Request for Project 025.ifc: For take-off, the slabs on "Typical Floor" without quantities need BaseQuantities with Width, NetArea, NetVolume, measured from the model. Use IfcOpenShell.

First a look at what the model holds.

```python
import ifcopenshell
import ifcopenshell.util.element
import ifcopenshell.util.unit

model = ifcopenshell.open("Project 025.ifc")
print(model.schema)
for unit_type in ("LENGTHUNIT", "AREAUNIT", "VOLUMEUNIT"):
    print(unit_type, ifcopenshell.util.unit.calculate_unit_scale(model, unit_type))
storey = next(s for s in model.by_type("IfcBuildingStorey") if s.Name == "Typical Floor")
slabs = [e for e in ifcopenshell.util.element.get_decomposition(storey) if e.is_a("IfcSlab")]
for e in sorted(slabs, key=lambda e: e.id()):
    print(e.id(), e.is_a(), e.Name, list(ifcopenshell.util.element.get_psets(e, qtos_only=True)), sep=" | ")
```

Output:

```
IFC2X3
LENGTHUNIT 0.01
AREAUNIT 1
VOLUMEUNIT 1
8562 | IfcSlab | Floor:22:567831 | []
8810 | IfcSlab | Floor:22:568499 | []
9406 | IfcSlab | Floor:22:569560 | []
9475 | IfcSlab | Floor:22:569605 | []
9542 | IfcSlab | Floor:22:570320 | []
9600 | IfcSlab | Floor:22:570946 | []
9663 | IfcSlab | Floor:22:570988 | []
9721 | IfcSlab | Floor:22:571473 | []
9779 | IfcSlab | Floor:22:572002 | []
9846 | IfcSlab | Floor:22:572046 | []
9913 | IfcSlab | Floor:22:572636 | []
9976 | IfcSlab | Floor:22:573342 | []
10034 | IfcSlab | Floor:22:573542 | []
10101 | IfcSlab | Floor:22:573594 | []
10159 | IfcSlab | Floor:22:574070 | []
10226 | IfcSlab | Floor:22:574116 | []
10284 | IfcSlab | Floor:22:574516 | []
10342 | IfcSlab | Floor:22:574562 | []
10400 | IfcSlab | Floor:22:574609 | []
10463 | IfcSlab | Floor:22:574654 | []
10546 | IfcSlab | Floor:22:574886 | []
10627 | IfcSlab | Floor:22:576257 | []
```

```python
import ifcopenshell
import ifcopenshell.api.pset
import ifcopenshell.geom
import ifcopenshell.util.element
import ifcopenshell.util.shape
import ifcopenshell.util.unit

model = ifcopenshell.open("Project 025.ifc")
unit_scale = ifcopenshell.util.unit.calculate_unit_scale(model)
area_scale = ifcopenshell.util.unit.calculate_unit_scale(model, "AREAUNIT")
volume_scale = ifcopenshell.util.unit.calculate_unit_scale(model, "VOLUMEUNIT")
settings = ifcopenshell.geom.settings()

storey = next(s for s in model.by_type("IfcBuildingStorey") if s.Name == "Typical Floor")
slabs = [e for e in ifcopenshell.util.element.get_decomposition(storey) if e.is_a("IfcSlab")]

for e in sorted(slabs, key=lambda e: e.id()):
    if ifcopenshell.util.element.get_psets(e, qtos_only=True, should_inherit=False):
        continue
    # Geometry comes back in metres, in the element's own axes.
    shape = ifcopenshell.geom.create_shape(settings, e)
    values = {
        "Width": ifcopenshell.util.shape.get_z(shape.geometry) / unit_scale,
        "NetArea": ifcopenshell.util.shape.get_footprint_area(shape.geometry) / area_scale,
        "NetVolume": ifcopenshell.util.shape.get_volume(shape.geometry) / volume_scale,
    }
    qto = ifcopenshell.api.pset.add_qto(model, product=e, name="BaseQuantities")
    ifcopenshell.api.pset.edit_qto(model, qto=qto, properties=values)
    print(e.id(), {k: round(v, 3) for k, v in values.items()})

model.write("Project 025-out.ifc")
```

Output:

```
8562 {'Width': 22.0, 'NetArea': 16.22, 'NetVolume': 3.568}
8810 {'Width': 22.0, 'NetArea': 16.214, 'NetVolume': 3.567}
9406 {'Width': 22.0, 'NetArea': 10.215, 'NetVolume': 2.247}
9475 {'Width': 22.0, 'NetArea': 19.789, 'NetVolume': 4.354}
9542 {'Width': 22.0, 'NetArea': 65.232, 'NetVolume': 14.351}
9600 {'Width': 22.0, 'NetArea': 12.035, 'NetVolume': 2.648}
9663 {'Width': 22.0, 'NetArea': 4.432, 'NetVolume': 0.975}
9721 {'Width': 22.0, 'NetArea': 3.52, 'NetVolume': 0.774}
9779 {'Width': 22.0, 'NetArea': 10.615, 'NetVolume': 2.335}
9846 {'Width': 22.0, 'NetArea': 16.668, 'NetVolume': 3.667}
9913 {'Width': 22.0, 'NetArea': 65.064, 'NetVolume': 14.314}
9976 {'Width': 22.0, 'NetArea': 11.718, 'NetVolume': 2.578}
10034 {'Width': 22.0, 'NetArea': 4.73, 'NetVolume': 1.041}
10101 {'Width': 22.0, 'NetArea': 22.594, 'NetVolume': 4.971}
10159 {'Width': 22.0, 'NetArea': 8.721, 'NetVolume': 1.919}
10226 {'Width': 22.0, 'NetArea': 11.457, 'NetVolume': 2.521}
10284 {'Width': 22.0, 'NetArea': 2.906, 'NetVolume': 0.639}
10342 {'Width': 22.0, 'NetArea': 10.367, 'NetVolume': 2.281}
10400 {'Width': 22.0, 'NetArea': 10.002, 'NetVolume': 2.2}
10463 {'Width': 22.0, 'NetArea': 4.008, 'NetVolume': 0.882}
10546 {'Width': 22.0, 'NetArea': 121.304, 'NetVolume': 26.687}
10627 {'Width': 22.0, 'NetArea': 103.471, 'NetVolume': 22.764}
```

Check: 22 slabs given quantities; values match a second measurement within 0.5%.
